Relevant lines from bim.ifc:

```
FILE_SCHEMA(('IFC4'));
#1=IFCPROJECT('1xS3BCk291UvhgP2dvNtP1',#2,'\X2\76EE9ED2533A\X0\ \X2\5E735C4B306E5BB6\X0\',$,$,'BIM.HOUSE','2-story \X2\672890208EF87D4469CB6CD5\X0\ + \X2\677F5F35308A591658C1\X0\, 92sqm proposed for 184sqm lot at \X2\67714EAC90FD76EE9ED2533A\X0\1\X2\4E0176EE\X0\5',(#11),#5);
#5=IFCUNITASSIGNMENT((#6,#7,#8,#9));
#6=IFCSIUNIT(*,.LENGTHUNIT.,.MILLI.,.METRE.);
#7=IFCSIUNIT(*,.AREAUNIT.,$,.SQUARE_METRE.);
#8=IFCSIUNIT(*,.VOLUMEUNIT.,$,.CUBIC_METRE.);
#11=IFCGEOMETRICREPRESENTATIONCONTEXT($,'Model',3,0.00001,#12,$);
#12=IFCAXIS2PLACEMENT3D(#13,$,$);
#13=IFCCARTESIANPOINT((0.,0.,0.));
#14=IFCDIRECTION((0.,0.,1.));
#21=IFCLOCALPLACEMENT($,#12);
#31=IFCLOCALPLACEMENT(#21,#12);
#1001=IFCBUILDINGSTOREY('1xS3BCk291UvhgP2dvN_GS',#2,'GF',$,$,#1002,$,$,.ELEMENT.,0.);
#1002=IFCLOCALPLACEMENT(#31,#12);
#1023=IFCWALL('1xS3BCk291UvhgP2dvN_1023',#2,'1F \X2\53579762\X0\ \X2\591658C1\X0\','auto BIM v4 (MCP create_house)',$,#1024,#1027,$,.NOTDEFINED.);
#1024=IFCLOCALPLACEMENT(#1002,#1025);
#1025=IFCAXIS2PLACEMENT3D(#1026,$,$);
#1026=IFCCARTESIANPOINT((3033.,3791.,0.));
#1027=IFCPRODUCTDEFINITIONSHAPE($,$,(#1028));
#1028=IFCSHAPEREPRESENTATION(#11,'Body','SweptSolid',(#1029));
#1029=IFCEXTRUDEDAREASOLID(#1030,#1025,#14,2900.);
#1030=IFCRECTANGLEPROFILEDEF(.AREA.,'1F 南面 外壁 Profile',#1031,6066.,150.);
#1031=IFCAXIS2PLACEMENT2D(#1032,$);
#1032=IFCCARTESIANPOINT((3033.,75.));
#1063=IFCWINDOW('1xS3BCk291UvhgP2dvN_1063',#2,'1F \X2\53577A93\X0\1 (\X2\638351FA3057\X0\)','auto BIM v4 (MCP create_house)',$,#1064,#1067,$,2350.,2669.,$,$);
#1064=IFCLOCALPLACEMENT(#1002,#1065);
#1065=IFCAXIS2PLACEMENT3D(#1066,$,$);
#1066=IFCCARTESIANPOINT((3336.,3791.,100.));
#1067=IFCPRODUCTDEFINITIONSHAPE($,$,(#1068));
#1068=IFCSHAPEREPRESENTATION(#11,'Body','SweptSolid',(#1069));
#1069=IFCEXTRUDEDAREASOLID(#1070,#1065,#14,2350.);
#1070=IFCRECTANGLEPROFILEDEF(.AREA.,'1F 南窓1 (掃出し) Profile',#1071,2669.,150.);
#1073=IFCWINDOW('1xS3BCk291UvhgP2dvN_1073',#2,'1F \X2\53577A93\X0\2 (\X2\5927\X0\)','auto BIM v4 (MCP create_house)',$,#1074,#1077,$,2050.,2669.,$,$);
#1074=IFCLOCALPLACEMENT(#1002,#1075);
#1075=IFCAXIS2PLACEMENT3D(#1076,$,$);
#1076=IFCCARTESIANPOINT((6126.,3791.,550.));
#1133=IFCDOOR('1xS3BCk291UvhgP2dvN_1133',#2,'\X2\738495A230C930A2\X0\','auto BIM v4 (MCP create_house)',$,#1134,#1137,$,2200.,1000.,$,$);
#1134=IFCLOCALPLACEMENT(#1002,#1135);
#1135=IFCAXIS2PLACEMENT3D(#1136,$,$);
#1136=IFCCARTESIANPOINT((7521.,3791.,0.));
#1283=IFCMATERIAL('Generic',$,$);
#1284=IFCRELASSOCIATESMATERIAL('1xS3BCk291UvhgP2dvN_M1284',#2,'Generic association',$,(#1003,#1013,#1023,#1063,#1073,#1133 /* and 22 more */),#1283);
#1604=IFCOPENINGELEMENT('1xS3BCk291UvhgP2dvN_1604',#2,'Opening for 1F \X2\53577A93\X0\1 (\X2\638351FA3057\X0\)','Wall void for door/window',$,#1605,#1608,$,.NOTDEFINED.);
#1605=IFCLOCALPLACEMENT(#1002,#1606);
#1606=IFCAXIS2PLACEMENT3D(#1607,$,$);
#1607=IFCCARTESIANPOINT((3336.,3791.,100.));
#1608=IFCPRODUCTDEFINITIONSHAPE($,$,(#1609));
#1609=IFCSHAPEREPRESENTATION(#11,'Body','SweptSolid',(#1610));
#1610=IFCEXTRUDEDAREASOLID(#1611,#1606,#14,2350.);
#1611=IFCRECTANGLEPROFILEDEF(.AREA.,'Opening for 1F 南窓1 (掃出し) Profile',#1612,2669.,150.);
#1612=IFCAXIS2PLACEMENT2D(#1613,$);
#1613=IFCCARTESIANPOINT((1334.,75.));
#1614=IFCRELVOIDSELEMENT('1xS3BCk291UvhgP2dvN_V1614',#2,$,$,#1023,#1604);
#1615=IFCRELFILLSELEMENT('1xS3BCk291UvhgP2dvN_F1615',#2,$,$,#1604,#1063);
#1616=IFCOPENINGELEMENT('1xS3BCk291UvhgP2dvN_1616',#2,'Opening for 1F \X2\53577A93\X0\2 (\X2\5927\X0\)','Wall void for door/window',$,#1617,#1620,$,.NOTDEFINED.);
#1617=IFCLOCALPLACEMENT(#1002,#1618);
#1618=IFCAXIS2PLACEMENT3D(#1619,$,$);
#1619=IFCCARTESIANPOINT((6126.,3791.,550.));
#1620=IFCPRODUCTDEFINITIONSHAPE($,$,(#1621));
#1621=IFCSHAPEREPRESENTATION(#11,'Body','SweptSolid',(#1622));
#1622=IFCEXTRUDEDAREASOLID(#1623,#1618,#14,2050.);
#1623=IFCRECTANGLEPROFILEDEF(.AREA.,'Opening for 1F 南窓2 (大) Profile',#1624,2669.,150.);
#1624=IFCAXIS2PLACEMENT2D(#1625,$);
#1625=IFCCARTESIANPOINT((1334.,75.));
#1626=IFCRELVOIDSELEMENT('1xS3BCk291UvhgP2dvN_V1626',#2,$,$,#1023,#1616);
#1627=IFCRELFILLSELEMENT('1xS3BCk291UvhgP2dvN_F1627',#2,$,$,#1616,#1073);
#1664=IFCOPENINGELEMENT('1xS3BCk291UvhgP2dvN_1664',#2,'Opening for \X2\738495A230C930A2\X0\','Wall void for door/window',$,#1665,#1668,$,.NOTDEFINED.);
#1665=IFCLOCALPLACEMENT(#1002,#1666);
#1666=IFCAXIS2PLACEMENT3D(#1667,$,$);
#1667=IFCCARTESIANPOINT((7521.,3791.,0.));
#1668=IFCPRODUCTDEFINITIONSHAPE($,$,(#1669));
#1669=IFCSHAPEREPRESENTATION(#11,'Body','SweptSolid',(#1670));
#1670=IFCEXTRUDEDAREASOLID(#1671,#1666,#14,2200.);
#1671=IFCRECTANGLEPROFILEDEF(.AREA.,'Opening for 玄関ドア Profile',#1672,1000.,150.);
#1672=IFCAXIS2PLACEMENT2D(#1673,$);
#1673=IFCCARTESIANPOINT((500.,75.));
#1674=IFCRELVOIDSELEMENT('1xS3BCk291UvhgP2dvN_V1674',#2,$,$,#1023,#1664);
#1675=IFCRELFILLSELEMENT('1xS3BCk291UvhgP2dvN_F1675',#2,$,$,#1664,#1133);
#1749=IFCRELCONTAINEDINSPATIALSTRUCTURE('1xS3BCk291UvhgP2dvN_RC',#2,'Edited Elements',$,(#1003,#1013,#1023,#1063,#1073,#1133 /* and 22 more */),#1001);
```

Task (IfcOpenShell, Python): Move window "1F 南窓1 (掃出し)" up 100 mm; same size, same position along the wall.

```python
import numpy as np
import ifcopenshell
import ifcopenshell.api.geometry
import ifcopenshell.util.placement
import ifcopenshell.util.unit

model = ifcopenshell.open("bim.ifc")
unit_scale = ifcopenshell.util.unit.calculate_unit_scale(model)

window = model.by_guid("1xS3BCk291UvhgP2dvN_1063")
opening = window.FillsVoids[0].RelatingOpeningElement
dz = 0.1 / unit_scale

shift = np.array([0.0, 0.0, dz])
# The window is not placed relative to its opening, so move both.
for product in (opening, window):
    matrix = ifcopenshell.util.placement.get_local_placement(product.ObjectPlacement)
    matrix[:3, 3] += shift
    ifcopenshell.api.geometry.edit_object_placement(model, product=product, matrix=matrix, is_si=False)

print(f"moved by {dz * unit_scale:+.3f} m")

model.write("bim_updated.ifc")
```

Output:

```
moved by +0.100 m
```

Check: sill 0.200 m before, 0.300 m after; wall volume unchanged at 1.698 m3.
